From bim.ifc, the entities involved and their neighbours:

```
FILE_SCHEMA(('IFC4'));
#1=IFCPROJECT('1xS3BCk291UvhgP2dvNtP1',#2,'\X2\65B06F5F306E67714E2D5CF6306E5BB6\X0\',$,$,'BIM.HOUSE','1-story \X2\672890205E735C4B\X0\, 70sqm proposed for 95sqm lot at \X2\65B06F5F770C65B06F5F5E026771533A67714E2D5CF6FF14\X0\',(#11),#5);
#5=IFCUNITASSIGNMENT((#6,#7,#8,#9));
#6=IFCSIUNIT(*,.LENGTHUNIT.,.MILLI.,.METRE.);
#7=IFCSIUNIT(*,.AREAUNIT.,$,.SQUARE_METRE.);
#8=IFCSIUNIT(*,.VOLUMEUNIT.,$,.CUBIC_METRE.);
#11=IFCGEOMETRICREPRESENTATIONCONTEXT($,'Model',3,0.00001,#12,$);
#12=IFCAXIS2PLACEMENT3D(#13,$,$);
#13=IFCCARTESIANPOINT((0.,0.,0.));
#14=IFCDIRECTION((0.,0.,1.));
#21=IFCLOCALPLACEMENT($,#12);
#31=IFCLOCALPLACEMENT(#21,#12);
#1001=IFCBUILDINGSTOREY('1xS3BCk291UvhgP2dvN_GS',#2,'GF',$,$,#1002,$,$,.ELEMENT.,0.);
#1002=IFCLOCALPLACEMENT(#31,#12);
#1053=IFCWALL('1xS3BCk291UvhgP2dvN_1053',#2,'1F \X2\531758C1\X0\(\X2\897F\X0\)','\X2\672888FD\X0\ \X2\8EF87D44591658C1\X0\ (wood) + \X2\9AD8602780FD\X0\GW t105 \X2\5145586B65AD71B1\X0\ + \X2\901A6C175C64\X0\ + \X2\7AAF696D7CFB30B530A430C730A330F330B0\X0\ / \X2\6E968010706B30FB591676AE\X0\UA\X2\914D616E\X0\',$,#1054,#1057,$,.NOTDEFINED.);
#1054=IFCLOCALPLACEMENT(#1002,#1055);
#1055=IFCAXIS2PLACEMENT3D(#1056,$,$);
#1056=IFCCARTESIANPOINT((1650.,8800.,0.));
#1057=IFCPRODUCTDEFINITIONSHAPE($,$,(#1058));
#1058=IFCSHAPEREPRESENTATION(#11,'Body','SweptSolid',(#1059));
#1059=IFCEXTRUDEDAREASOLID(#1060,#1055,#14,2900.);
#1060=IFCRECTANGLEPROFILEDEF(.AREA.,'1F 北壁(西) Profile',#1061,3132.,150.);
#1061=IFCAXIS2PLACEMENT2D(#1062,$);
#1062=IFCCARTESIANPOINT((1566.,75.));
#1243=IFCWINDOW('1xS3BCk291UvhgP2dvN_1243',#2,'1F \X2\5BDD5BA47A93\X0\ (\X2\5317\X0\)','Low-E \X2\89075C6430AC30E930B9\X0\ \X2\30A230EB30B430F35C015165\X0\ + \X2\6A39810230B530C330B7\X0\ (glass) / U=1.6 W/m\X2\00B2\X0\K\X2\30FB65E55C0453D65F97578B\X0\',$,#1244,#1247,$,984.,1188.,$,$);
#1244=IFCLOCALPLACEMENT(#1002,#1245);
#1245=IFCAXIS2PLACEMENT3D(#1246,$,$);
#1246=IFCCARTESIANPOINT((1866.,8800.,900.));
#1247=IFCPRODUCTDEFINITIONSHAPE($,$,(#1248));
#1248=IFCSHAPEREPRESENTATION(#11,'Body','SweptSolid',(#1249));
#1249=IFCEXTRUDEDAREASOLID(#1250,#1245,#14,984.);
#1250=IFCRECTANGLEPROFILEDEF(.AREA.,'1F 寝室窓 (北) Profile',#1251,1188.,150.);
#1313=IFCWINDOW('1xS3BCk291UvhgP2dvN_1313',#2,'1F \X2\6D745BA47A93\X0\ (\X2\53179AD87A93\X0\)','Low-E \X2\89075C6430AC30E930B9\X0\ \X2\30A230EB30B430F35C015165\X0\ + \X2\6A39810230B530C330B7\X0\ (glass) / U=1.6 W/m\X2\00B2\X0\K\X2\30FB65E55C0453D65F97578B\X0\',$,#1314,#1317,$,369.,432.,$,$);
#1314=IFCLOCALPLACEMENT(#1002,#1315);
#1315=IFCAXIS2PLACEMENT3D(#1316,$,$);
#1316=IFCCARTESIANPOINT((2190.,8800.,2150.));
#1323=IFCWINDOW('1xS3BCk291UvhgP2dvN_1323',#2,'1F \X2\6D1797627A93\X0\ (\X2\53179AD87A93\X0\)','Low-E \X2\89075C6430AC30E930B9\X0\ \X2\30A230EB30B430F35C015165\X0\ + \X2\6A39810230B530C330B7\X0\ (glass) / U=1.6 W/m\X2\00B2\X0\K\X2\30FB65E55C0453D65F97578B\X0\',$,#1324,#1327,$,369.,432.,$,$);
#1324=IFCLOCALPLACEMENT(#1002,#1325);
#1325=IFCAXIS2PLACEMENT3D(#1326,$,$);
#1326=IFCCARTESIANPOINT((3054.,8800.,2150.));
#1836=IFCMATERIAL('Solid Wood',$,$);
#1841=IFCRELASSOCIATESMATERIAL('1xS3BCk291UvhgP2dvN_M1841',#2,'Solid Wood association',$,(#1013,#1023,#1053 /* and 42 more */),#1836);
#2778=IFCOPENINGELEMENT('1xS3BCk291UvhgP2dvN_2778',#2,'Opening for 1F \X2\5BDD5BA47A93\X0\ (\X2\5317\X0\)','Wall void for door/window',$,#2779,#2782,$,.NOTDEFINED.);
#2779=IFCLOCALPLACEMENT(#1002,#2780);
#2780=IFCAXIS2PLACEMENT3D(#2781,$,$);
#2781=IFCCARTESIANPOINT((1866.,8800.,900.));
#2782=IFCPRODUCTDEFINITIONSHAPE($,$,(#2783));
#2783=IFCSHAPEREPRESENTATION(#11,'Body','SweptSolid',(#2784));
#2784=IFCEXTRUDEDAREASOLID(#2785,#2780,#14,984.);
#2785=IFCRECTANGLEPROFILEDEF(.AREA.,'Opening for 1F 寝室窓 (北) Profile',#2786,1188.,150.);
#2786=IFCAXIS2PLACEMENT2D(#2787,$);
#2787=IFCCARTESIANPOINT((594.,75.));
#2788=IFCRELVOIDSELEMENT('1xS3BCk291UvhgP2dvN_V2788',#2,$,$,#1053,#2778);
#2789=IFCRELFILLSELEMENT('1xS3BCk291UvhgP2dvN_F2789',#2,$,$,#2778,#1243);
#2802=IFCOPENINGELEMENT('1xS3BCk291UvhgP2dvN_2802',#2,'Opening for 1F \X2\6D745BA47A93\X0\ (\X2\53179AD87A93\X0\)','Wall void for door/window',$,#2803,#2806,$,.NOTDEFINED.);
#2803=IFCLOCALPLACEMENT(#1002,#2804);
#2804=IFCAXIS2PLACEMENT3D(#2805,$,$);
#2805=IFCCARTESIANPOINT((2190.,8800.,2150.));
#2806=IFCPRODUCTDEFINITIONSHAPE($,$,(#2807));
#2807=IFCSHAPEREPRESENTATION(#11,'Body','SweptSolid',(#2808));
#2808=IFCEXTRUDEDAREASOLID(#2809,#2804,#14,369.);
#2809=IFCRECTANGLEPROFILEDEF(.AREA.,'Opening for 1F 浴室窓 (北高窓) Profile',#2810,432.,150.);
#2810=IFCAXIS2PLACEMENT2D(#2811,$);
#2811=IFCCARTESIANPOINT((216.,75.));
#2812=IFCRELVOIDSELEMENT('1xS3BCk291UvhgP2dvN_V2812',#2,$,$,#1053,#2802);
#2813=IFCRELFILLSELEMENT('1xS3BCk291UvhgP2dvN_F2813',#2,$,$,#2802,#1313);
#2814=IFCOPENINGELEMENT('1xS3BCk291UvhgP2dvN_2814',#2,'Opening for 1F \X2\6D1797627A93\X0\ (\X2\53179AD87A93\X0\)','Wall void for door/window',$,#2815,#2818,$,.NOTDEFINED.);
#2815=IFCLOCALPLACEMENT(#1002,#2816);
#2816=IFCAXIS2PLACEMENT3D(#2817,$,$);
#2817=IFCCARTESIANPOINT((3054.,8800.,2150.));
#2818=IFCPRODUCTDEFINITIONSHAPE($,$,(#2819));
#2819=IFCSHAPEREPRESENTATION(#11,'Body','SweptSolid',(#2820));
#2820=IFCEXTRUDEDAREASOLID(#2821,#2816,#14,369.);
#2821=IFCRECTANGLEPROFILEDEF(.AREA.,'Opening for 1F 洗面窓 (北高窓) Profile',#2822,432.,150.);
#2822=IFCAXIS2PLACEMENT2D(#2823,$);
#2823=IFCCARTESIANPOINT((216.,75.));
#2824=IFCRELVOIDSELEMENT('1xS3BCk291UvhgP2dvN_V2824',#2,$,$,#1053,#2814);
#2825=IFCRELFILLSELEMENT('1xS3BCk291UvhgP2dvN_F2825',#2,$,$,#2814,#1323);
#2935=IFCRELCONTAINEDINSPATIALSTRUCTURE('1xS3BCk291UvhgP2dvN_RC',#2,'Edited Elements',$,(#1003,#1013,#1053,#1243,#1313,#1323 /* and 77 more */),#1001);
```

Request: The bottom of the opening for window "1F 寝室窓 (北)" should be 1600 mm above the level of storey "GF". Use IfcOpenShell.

```python
import numpy as np
import ifcopenshell
import ifcopenshell.api.geometry
import ifcopenshell.geom
import ifcopenshell.util.element
import ifcopenshell.util.placement
import ifcopenshell.util.shape
import ifcopenshell.util.unit

model = ifcopenshell.open("bim.ifc")
unit_scale = ifcopenshell.util.unit.calculate_unit_scale(model)

window = model.by_guid("1xS3BCk291UvhgP2dvN_1243")
opening = window.FillsVoids[0].RelatingOpeningElement
storey = ifcopenshell.util.element.get_container(window, ifc_class="IfcBuildingStorey")
level = ifcopenshell.util.placement.get_local_placement(storey.ObjectPlacement)[2, 3]

# The opening's origin need not be at the sill, so measure its lowest point.
shape = ifcopenshell.geom.create_shape(ifcopenshell.geom.settings(), opening)
bottom = ifcopenshell.util.shape.get_shape_bottom_elevation(shape, shape.geometry) / unit_scale
dz = level + 1.6 / unit_scale - bottom

shift = np.array([0.0, 0.0, dz])
# The window is not placed relative to its opening, so move both.
for product in (opening, window):
    matrix = ifcopenshell.util.placement.get_local_placement(product.ObjectPlacement)
    matrix[:3, 3] += shift
    ifcopenshell.api.geometry.edit_object_placement(model, product=product, matrix=matrix, is_si=False)

print(f"moved by {dz * unit_scale:+.3f} m")

model.write("bim_updated.ifc")
```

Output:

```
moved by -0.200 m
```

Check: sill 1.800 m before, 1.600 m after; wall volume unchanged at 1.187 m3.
